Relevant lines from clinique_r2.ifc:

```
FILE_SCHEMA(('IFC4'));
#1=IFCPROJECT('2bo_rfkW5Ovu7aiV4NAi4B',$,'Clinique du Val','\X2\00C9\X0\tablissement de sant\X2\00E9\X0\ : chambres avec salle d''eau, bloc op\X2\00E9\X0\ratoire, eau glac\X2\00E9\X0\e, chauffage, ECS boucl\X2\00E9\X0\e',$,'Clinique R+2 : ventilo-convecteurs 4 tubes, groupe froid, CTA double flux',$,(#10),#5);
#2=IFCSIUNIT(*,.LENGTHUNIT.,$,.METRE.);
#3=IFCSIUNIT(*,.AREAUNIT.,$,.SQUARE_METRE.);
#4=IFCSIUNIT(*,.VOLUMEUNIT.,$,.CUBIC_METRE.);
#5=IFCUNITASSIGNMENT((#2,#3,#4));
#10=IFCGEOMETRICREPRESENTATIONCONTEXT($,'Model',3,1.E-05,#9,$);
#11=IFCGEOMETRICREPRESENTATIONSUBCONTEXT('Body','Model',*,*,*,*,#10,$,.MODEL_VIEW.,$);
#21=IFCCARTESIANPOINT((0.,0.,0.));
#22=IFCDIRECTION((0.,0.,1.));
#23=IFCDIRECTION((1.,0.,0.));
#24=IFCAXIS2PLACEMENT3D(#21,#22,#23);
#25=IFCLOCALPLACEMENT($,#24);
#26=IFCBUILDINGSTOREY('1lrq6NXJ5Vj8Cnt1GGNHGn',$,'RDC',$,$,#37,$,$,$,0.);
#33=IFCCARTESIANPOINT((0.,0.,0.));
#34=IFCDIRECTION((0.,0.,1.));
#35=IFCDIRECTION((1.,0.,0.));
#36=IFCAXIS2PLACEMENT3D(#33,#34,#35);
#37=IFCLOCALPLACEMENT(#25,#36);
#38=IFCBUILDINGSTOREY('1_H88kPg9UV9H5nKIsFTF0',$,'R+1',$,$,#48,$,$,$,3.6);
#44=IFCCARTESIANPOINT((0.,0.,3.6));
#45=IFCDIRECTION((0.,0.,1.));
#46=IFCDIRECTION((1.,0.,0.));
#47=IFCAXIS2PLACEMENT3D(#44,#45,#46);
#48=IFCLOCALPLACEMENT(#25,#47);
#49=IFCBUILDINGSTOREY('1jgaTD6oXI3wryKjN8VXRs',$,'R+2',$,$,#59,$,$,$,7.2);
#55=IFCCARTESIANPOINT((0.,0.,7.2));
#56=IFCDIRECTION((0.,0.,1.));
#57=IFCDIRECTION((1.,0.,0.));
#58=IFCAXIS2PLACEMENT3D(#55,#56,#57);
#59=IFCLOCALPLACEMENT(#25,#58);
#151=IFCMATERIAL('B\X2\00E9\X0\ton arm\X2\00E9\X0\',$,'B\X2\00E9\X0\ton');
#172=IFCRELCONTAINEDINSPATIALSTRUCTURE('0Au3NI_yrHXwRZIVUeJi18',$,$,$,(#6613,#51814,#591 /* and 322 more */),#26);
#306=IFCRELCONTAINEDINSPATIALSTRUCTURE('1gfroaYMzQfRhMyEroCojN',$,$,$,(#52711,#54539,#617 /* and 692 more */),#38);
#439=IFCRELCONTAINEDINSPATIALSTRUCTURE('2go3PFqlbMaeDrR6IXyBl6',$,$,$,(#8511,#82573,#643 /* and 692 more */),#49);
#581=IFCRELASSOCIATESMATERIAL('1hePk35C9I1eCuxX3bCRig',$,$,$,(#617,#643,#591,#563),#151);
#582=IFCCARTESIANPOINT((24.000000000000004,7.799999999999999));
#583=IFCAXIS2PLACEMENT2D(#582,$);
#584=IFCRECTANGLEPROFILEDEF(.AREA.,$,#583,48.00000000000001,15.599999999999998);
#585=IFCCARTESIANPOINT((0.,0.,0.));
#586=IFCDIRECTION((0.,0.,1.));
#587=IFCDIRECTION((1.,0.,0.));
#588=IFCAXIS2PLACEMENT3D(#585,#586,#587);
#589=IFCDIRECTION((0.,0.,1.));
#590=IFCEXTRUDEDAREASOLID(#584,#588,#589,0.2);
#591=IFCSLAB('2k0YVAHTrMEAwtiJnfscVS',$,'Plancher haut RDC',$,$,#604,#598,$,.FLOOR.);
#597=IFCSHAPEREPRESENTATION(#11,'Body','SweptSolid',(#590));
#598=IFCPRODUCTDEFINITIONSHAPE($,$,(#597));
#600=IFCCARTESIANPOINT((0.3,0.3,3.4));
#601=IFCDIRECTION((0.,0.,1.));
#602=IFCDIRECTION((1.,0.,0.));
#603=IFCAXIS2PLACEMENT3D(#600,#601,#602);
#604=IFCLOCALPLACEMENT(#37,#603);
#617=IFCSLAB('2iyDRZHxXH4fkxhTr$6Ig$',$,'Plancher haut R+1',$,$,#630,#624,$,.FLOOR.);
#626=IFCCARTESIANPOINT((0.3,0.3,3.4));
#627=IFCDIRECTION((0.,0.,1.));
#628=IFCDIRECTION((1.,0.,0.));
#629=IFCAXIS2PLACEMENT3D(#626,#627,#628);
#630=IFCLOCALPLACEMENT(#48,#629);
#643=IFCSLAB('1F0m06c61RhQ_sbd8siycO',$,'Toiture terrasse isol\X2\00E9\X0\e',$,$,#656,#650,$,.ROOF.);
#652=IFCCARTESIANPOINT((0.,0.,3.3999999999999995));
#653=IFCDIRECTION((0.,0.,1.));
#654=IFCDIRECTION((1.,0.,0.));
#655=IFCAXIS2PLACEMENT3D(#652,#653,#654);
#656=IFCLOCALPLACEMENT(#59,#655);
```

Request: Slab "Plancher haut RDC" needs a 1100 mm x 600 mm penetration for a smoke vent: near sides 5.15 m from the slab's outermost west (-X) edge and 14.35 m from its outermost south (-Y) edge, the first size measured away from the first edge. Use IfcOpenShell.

```python
import numpy as np
import ifcopenshell
import ifcopenshell.api.feature
import ifcopenshell.api.geometry
import ifcopenshell.api.root
import ifcopenshell.geom
import ifcopenshell.util.placement
import ifcopenshell.util.representation
import ifcopenshell.util.shape
import ifcopenshell.util.unit

model = ifcopenshell.open("clinique_r2.ifc")
unit_scale = ifcopenshell.util.unit.calculate_unit_scale(model)
settings = ifcopenshell.geom.settings()


def volume(element):
    """Net volume in cubic metres, openings subtracted."""
    shape = ifcopenshell.geom.create_shape(settings, element)
    return ifcopenshell.util.shape.get_volume(shape.geometry)


slab = model.by_guid("2k0YVAHTrMEAwtiJnfscVS")
before = volume(slab)

# Extent in the slab's own axes, in metres. The edges named are its -X and -Y sides.
slab_shape = ifcopenshell.geom.create_shape(settings, slab)
vertices = ifcopenshell.util.shape.get_vertices(slab_shape.geometry)
x_min, y_min, bottom = vertices.min(axis=0)
top = vertices[:, 2].max()

opening = ifcopenshell.api.root.create_entity(model, ifc_class="IfcOpeningElement", name="Smoke vent opening", predefined_type="OPENING")
context = ifcopenshell.util.representation.get_context(model, "Model", "Body", "MODEL_VIEW")
width, depth = 1.1, 0.6
outline = [(0.0, 0.0), (width, 0.0), (width, depth), (0.0, depth), (0.0, 0.0)]
# Overshoot both faces by 50 mm so the cut is clean.
shape = ifcopenshell.api.geometry.add_slab_representation(
    model, context=context, depth=top - bottom + 0.1, polyline=outline
)
ifcopenshell.api.geometry.assign_representation(model, product=opening, representation=shape)

matrix = ifcopenshell.util.placement.get_local_placement(slab.ObjectPlacement)
matrix[:, 3] = matrix @ np.append(np.array([x_min + 5.15, y_min + 14.35, bottom - 0.05]) / unit_scale, 1.0)
ifcopenshell.api.geometry.edit_object_placement(model, product=opening, matrix=matrix, is_si=False)
ifcopenshell.api.feature.add_feature(model, feature=opening, element=slab)

after = volume(slab)

print(f"slab volume {before:.3f} -> {after:.3f} m3")

model.write("clinique_r2_updated.ifc")
```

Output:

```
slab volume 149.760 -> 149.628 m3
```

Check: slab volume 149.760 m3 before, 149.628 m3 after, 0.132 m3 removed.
